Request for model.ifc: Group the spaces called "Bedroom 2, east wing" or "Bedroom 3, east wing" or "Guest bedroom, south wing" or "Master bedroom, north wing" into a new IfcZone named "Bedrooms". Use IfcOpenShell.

First a look at what the model holds.

```python
import ifcopenshell

model = ifcopenshell.open("model.ifc")
print(model.schema)
seen = {}
for space in model.by_type("IfcSpace"):
    seen[space.LongName] = seen.get(space.LongName, 0) + 1
for name, count in sorted(seen.items(), key=str):
    print(count, "x", name)
print("zones:", [z.Name for z in model.by_type("IfcZone")][:20])
```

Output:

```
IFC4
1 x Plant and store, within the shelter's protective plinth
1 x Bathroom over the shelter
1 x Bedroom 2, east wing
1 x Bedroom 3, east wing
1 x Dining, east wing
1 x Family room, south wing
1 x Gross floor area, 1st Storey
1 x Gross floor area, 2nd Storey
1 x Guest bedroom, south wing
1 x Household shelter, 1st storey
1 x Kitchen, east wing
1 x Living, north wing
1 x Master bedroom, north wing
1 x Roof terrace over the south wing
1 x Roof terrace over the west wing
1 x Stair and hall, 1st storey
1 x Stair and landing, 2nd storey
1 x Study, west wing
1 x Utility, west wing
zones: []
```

```python
import ifcopenshell
import ifcopenshell.api.group
import ifcopenshell.api.root

model = ifcopenshell.open("model.ifc")

names = {"Bedroom 2, east wing", "Bedroom 3, east wing", "Guest bedroom, south wing", "Master bedroom, north wing"}
spaces = [s for s in model.by_type("IfcSpace") if s.LongName in names]

zone = ifcopenshell.api.root.create_entity(model, ifc_class="IfcZone", name="Bedrooms")
ifcopenshell.api.group.assign_group(model, products=spaces, group=zone)
print(len(spaces), "spaces in", zone.Name)

model.write("model_updated.ifc")
```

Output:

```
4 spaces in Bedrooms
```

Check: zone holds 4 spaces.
